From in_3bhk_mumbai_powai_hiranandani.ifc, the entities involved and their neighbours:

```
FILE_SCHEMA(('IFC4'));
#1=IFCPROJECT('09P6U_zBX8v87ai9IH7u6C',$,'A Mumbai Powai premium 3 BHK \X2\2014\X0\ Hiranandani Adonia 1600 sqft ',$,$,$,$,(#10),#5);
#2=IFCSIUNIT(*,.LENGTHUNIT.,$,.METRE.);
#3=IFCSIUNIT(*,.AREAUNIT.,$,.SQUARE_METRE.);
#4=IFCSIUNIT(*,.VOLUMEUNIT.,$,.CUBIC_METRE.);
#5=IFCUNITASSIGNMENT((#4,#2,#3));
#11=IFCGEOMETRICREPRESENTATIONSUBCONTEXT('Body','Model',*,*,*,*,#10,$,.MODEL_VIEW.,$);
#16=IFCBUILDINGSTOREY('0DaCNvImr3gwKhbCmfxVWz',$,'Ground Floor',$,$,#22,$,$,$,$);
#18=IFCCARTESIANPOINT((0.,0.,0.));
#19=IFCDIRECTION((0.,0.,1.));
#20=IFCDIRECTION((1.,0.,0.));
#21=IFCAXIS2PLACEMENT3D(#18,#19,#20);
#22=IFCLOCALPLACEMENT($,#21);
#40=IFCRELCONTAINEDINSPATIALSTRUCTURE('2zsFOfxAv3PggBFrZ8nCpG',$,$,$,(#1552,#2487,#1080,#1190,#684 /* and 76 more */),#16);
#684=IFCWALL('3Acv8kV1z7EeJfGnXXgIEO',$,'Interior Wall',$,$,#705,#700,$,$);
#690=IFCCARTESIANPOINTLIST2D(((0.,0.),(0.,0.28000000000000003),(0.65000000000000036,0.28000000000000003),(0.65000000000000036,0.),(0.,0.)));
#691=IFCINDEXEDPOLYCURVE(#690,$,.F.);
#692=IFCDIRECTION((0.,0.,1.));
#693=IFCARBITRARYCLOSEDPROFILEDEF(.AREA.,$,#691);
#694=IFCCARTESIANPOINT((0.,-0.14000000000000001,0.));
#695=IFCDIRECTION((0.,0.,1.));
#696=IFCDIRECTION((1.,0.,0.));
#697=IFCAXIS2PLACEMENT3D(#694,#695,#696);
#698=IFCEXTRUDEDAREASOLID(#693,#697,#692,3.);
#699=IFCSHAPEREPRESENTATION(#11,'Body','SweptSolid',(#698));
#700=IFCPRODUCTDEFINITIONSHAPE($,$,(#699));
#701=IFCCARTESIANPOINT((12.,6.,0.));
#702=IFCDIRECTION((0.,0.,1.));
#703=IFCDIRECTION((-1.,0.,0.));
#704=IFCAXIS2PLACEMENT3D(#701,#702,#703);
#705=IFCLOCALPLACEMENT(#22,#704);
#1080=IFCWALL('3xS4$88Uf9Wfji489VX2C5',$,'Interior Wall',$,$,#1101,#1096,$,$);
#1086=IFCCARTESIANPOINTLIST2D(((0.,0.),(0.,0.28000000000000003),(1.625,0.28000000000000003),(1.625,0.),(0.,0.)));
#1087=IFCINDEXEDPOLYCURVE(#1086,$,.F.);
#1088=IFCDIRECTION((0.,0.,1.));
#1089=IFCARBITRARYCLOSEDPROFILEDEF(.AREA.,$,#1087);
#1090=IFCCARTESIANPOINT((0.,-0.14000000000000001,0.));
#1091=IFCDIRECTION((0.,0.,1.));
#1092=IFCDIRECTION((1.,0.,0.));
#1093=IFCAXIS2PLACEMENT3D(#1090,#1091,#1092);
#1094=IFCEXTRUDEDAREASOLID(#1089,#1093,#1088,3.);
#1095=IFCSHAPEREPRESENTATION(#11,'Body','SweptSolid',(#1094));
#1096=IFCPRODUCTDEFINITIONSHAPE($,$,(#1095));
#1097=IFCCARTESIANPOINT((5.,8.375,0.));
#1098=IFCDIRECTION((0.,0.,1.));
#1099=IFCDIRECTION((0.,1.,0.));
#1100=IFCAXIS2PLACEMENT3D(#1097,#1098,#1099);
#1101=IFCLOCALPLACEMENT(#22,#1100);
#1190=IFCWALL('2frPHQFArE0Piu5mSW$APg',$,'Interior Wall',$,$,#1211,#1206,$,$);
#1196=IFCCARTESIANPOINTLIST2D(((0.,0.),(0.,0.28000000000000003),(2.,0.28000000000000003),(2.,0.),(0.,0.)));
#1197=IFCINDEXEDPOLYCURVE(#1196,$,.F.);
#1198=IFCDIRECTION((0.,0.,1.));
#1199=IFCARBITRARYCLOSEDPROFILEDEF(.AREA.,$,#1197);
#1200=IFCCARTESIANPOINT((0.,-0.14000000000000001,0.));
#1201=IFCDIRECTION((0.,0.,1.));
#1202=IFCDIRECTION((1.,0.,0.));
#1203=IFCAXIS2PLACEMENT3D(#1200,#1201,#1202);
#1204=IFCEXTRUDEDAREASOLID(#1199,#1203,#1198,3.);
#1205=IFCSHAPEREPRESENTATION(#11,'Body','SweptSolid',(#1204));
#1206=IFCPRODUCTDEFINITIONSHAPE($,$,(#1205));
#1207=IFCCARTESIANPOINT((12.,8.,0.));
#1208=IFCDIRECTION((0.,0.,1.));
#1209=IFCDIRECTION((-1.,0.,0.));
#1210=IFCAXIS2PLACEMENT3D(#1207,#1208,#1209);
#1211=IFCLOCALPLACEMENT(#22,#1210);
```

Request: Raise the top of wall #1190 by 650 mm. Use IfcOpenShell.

```python
import ifcopenshell
import ifcopenshell.geom
import ifcopenshell.util.representation
import ifcopenshell.util.shape
import ifcopenshell.util.unit

model = ifcopenshell.open("in_3bhk_mumbai_powai_hiranandani.ifc")
unit_scale = ifcopenshell.util.unit.calculate_unit_scale(model)
settings = ifcopenshell.geom.settings()


def volume(element):
    """Net volume in cubic metres, openings subtracted."""
    shape = ifcopenshell.geom.create_shape(settings, element)
    return ifcopenshell.util.shape.get_volume(shape.geometry)


wall = model.by_id(1190)
before = volume(wall)

body = ifcopenshell.util.representation.get_representation(wall, "Model", "Body")
solid = body.Items[0]
old_height = solid.Depth
solid.Depth += 0.65 / unit_scale
after = volume(wall)

print(f"height {old_height:g} -> {solid.Depth:g}, volume {before:.3f} -> {after:.3f} m3")

model.write("in_3bhk_mumbai_powai_hiranandani-out.ifc")
```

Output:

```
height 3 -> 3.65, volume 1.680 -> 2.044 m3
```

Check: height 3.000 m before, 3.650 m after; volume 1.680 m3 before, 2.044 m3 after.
